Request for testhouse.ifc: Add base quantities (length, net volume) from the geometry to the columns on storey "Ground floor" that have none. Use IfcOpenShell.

First a look at what the model holds.

```python
import ifcopenshell
import ifcopenshell.util.element
import ifcopenshell.util.unit

model = ifcopenshell.open("testhouse.ifc")
print(model.schema)
for unit_type in ("LENGTHUNIT", "AREAUNIT", "VOLUMEUNIT"):
    print(unit_type, ifcopenshell.util.unit.calculate_unit_scale(model, unit_type))
storey = next(s for s in model.by_type("IfcBuildingStorey") if s.Name == "Ground floor")
columns = [e for e in ifcopenshell.util.element.get_decomposition(storey) if e.is_a("IfcColumn")]
for e in sorted(columns, key=lambda e: e.id()):
    print(e.id(), e.is_a(), e.Name, list(ifcopenshell.util.element.get_psets(e, qtos_only=True)), sep=" | ")
```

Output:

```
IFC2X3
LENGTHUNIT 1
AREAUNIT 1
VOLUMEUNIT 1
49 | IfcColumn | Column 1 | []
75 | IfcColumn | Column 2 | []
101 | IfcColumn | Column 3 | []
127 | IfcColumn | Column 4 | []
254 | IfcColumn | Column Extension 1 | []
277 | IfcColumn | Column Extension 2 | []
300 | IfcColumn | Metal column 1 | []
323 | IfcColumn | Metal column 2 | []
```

```python
import ifcopenshell
import ifcopenshell.api.pset
import ifcopenshell.geom
import ifcopenshell.util.element
import ifcopenshell.util.shape
import ifcopenshell.util.unit

model = ifcopenshell.open("testhouse.ifc")
unit_scale = ifcopenshell.util.unit.calculate_unit_scale(model)
volume_scale = ifcopenshell.util.unit.calculate_unit_scale(model, "VOLUMEUNIT")
settings = ifcopenshell.geom.settings()

storey = next(s for s in model.by_type("IfcBuildingStorey") if s.Name == "Ground floor")
columns = [e for e in ifcopenshell.util.element.get_decomposition(storey) if e.is_a("IfcColumn")]

for e in sorted(columns, key=lambda e: e.id()):
    if ifcopenshell.util.element.get_psets(e, qtos_only=True, should_inherit=False):
        continue
    # Geometry comes back in metres, in the element's own axes.
    shape = ifcopenshell.geom.create_shape(settings, e)
    values = {
        "Length": ifcopenshell.util.shape.get_z(shape.geometry) / unit_scale,
        "NetVolume": ifcopenshell.util.shape.get_volume(shape.geometry) / volume_scale,
    }
    qto = ifcopenshell.api.pset.add_qto(model, product=e, name="BaseQuantities")
    ifcopenshell.api.pset.edit_qto(model, qto=qto, properties=values)
    print(e.id(), {k: round(v, 3) for k, v in values.items()})

model.write("testhouse_edited.ifc")
```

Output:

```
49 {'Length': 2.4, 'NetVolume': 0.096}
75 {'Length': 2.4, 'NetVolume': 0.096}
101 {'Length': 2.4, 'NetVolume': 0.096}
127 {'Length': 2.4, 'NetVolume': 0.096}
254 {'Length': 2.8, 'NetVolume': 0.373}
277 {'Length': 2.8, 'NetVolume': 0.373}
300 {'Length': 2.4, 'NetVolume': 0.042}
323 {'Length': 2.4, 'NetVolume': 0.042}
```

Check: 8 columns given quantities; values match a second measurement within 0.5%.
